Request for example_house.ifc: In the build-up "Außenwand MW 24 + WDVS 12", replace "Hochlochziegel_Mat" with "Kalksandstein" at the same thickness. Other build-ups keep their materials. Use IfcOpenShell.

First a look at what the model holds.

```python
import ifcopenshell
import ifcopenshell.util.element

model = ifcopenshell.open("example_house.ifc")
print(model.schema)
for layer_set in model.by_type("IfcMaterialLayerSet"):
    if layer_set.LayerSetName == "Außenwand MW 24 + WDVS 12":
        for layer in layer_set.MaterialLayers:
            print(layer.id(), layer.Material and layer.Material.Name, layer.LayerThickness, sep=" | ")
        print(len(ifcopenshell.util.element.get_elements_by_material(model, layer_set)), "elements and types use it")
print(sorted(m.Name for m in model.by_type("IfcMaterial") if m.Name)[:60])
```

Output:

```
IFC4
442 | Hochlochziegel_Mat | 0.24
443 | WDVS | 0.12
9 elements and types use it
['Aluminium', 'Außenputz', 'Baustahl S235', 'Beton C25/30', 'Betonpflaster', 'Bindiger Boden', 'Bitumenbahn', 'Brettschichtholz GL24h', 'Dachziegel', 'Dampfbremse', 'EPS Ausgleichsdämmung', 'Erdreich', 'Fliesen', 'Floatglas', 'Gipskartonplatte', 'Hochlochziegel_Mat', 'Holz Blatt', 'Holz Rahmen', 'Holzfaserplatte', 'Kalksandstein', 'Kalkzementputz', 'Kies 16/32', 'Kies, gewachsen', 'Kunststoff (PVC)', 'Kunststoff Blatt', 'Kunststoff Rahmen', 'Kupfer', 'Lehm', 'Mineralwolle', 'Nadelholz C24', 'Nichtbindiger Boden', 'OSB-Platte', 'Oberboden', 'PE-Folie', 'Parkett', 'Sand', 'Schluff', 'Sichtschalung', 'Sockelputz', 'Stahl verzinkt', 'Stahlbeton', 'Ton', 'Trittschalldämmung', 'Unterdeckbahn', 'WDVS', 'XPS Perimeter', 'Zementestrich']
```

```python
import ifcopenshell
import ifcopenshell.api.material

model = ifcopenshell.open("example_house.ifc")

layer_set = next(s for s in model.by_type("IfcMaterialLayerSet") if s.LayerSetName == "Außenwand MW 24 + WDVS 12")
layer = next(l for l in layer_set.MaterialLayers if l.Material and l.Material.Name == "Hochlochziegel_Mat")
material = next(m for m in model.by_type("IfcMaterial") if m.Name == "Kalksandstein")

# Point this one layer at the other material; renaming the old one would change it everywhere.
ifcopenshell.api.material.edit_layer(model, layer=layer, attributes={"Name": material.Name}, material=material)

print([l.Material.Name if l.Material else None for l in layer_set.MaterialLayers])

model.write("example_house_edited.ifc")
```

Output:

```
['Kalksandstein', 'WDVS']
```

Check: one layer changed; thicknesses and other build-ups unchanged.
